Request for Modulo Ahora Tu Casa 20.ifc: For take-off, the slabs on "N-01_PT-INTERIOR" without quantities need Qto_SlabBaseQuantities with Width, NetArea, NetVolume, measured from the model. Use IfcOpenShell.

First a look at what the model holds.

```python
import ifcopenshell
import ifcopenshell.util.element
import ifcopenshell.util.unit

model = ifcopenshell.open("Modulo Ahora Tu Casa 20.ifc")
print(model.schema)
for unit_type in ("LENGTHUNIT", "AREAUNIT", "VOLUMEUNIT"):
    print(unit_type, ifcopenshell.util.unit.calculate_unit_scale(model, unit_type))
storey = next(s for s in model.by_type("IfcBuildingStorey") if s.Name == "N-01_PT-INTERIOR")
slabs = [e for e in ifcopenshell.util.element.get_decomposition(storey) if e.is_a("IfcSlab")]
for e in sorted(slabs, key=lambda e: e.id()):
    print(e.id(), e.is_a(), e.Name, list(ifcopenshell.util.element.get_psets(e, qtos_only=True)), sep=" | ")
```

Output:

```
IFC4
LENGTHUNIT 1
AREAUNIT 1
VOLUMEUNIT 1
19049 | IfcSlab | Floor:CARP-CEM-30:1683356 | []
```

```python
import ifcopenshell
import ifcopenshell.api.pset
import ifcopenshell.geom
import ifcopenshell.util.element
import ifcopenshell.util.shape
import ifcopenshell.util.unit

model = ifcopenshell.open("Modulo Ahora Tu Casa 20.ifc")
unit_scale = ifcopenshell.util.unit.calculate_unit_scale(model)
area_scale = ifcopenshell.util.unit.calculate_unit_scale(model, "AREAUNIT")
volume_scale = ifcopenshell.util.unit.calculate_unit_scale(model, "VOLUMEUNIT")
settings = ifcopenshell.geom.settings()

storey = next(s for s in model.by_type("IfcBuildingStorey") if s.Name == "N-01_PT-INTERIOR")
slabs = [e for e in ifcopenshell.util.element.get_decomposition(storey) if e.is_a("IfcSlab")]

for e in sorted(slabs, key=lambda e: e.id()):
    if ifcopenshell.util.element.get_psets(e, qtos_only=True, should_inherit=False):
        continue
    # Geometry comes back in metres, in the element's own axes.
    shape = ifcopenshell.geom.create_shape(settings, e)
    values = {
        "Width": ifcopenshell.util.shape.get_z(shape.geometry) / unit_scale,
        "NetArea": ifcopenshell.util.shape.get_footprint_area(shape.geometry) / area_scale,
        "NetVolume": ifcopenshell.util.shape.get_volume(shape.geometry) / volume_scale,
    }
    qto = ifcopenshell.api.pset.add_qto(model, product=e, name="Qto_SlabBaseQuantities")
    ifcopenshell.api.pset.edit_qto(model, qto=qto, properties=values)
    print(e.id(), {k: round(v, 3) for k, v in values.items()})

model.write("Modulo Ahora Tu Casa 20-out.ifc")
```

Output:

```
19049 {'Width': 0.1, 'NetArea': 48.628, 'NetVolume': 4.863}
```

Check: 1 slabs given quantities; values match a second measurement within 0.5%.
